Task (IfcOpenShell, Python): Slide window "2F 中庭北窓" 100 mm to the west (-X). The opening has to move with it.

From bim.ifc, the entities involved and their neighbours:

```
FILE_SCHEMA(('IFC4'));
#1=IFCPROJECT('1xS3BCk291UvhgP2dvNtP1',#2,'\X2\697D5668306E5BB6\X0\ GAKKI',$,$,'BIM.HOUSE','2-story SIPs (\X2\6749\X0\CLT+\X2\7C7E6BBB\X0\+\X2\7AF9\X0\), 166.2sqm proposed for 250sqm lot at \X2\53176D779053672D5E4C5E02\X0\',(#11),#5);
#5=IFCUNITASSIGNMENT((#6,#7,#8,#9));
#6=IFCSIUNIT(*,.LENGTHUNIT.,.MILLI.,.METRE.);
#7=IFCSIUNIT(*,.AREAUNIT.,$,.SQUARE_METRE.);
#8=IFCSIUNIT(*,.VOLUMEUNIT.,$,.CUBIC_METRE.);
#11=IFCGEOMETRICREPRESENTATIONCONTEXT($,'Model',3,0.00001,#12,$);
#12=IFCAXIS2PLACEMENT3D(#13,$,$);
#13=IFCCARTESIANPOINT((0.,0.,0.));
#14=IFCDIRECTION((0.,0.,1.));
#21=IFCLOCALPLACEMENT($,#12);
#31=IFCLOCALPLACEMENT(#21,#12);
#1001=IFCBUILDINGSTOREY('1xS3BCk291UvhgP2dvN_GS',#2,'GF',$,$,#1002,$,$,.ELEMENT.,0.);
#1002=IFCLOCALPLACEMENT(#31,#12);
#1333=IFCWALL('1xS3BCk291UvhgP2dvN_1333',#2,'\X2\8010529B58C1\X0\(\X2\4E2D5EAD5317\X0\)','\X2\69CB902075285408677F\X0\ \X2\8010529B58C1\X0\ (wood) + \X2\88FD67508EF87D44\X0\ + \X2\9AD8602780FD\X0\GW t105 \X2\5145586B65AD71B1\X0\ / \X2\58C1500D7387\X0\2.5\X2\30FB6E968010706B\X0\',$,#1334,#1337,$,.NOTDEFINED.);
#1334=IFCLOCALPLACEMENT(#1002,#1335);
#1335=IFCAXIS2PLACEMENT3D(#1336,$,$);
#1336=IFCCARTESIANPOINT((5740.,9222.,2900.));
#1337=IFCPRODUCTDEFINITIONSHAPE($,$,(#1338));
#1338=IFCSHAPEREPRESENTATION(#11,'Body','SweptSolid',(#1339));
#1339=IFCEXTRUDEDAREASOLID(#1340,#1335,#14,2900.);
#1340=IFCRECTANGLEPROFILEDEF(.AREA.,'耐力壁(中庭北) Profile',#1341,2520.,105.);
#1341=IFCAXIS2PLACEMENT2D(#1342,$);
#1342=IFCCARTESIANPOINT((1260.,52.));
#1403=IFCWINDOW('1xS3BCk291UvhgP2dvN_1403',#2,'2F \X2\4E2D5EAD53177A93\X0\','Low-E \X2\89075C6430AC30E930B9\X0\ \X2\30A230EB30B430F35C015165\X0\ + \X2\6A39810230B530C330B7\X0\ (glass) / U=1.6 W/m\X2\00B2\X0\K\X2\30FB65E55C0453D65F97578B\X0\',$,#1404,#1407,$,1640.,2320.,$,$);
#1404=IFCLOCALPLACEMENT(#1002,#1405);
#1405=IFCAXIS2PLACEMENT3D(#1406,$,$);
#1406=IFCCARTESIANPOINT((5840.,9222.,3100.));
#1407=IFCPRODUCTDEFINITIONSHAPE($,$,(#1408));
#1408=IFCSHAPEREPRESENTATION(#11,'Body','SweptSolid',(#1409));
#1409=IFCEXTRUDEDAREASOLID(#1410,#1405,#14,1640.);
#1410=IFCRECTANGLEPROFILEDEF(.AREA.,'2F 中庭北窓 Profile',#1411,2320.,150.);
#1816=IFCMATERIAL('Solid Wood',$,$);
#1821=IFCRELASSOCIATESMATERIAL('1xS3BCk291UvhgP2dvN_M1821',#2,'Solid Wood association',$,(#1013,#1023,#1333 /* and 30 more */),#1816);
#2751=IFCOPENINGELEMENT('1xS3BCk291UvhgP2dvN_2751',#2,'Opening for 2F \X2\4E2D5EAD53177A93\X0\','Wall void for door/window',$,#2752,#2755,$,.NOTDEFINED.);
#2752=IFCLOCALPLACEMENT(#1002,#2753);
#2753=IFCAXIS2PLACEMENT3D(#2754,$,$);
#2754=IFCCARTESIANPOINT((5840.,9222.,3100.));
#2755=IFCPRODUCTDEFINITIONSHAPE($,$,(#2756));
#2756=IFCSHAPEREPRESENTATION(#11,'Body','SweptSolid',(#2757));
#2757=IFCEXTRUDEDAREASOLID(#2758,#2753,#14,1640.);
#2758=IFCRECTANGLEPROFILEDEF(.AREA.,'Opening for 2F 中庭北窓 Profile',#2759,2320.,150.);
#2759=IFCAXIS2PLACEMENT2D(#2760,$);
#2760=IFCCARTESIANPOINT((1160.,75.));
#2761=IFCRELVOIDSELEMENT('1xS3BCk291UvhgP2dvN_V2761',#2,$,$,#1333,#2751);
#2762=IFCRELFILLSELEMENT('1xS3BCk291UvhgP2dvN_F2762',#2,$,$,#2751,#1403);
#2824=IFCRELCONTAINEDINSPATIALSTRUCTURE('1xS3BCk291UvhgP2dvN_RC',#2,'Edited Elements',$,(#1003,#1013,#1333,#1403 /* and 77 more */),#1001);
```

```python
import ifcopenshell
import ifcopenshell.api.geometry
import ifcopenshell.util.placement
import ifcopenshell.util.unit

model = ifcopenshell.open("bim.ifc")
unit_scale = ifcopenshell.util.unit.calculate_unit_scale(model)

window = model.by_guid("1xS3BCk291UvhgP2dvN_1403")
opening = window.FillsVoids[0].RelatingOpeningElement
wall = opening.VoidsElements[0].RelatingBuildingElement

wall_matrix = ifcopenshell.util.placement.get_local_placement(wall.ObjectPlacement)
shift = wall_matrix[:3, 0] * -0.1 / unit_scale
before = ifcopenshell.util.placement.get_local_placement(window.ObjectPlacement)[:3, 3].copy()

# The window is not placed relative to its opening, so move both.
for product in (opening, window):
    matrix = ifcopenshell.util.placement.get_local_placement(product.ObjectPlacement)
    matrix[:3, 3] += shift
    ifcopenshell.api.geometry.edit_object_placement(model, product=product, matrix=matrix, is_si=False)

after = ifcopenshell.util.placement.get_local_placement(window.ObjectPlacement)[:3, 3]
print("window moved by", (after - before).round(3) + 0.0)

model.write("bim-out.ifc")
```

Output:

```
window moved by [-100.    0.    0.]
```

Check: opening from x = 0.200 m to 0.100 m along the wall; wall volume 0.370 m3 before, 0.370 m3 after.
